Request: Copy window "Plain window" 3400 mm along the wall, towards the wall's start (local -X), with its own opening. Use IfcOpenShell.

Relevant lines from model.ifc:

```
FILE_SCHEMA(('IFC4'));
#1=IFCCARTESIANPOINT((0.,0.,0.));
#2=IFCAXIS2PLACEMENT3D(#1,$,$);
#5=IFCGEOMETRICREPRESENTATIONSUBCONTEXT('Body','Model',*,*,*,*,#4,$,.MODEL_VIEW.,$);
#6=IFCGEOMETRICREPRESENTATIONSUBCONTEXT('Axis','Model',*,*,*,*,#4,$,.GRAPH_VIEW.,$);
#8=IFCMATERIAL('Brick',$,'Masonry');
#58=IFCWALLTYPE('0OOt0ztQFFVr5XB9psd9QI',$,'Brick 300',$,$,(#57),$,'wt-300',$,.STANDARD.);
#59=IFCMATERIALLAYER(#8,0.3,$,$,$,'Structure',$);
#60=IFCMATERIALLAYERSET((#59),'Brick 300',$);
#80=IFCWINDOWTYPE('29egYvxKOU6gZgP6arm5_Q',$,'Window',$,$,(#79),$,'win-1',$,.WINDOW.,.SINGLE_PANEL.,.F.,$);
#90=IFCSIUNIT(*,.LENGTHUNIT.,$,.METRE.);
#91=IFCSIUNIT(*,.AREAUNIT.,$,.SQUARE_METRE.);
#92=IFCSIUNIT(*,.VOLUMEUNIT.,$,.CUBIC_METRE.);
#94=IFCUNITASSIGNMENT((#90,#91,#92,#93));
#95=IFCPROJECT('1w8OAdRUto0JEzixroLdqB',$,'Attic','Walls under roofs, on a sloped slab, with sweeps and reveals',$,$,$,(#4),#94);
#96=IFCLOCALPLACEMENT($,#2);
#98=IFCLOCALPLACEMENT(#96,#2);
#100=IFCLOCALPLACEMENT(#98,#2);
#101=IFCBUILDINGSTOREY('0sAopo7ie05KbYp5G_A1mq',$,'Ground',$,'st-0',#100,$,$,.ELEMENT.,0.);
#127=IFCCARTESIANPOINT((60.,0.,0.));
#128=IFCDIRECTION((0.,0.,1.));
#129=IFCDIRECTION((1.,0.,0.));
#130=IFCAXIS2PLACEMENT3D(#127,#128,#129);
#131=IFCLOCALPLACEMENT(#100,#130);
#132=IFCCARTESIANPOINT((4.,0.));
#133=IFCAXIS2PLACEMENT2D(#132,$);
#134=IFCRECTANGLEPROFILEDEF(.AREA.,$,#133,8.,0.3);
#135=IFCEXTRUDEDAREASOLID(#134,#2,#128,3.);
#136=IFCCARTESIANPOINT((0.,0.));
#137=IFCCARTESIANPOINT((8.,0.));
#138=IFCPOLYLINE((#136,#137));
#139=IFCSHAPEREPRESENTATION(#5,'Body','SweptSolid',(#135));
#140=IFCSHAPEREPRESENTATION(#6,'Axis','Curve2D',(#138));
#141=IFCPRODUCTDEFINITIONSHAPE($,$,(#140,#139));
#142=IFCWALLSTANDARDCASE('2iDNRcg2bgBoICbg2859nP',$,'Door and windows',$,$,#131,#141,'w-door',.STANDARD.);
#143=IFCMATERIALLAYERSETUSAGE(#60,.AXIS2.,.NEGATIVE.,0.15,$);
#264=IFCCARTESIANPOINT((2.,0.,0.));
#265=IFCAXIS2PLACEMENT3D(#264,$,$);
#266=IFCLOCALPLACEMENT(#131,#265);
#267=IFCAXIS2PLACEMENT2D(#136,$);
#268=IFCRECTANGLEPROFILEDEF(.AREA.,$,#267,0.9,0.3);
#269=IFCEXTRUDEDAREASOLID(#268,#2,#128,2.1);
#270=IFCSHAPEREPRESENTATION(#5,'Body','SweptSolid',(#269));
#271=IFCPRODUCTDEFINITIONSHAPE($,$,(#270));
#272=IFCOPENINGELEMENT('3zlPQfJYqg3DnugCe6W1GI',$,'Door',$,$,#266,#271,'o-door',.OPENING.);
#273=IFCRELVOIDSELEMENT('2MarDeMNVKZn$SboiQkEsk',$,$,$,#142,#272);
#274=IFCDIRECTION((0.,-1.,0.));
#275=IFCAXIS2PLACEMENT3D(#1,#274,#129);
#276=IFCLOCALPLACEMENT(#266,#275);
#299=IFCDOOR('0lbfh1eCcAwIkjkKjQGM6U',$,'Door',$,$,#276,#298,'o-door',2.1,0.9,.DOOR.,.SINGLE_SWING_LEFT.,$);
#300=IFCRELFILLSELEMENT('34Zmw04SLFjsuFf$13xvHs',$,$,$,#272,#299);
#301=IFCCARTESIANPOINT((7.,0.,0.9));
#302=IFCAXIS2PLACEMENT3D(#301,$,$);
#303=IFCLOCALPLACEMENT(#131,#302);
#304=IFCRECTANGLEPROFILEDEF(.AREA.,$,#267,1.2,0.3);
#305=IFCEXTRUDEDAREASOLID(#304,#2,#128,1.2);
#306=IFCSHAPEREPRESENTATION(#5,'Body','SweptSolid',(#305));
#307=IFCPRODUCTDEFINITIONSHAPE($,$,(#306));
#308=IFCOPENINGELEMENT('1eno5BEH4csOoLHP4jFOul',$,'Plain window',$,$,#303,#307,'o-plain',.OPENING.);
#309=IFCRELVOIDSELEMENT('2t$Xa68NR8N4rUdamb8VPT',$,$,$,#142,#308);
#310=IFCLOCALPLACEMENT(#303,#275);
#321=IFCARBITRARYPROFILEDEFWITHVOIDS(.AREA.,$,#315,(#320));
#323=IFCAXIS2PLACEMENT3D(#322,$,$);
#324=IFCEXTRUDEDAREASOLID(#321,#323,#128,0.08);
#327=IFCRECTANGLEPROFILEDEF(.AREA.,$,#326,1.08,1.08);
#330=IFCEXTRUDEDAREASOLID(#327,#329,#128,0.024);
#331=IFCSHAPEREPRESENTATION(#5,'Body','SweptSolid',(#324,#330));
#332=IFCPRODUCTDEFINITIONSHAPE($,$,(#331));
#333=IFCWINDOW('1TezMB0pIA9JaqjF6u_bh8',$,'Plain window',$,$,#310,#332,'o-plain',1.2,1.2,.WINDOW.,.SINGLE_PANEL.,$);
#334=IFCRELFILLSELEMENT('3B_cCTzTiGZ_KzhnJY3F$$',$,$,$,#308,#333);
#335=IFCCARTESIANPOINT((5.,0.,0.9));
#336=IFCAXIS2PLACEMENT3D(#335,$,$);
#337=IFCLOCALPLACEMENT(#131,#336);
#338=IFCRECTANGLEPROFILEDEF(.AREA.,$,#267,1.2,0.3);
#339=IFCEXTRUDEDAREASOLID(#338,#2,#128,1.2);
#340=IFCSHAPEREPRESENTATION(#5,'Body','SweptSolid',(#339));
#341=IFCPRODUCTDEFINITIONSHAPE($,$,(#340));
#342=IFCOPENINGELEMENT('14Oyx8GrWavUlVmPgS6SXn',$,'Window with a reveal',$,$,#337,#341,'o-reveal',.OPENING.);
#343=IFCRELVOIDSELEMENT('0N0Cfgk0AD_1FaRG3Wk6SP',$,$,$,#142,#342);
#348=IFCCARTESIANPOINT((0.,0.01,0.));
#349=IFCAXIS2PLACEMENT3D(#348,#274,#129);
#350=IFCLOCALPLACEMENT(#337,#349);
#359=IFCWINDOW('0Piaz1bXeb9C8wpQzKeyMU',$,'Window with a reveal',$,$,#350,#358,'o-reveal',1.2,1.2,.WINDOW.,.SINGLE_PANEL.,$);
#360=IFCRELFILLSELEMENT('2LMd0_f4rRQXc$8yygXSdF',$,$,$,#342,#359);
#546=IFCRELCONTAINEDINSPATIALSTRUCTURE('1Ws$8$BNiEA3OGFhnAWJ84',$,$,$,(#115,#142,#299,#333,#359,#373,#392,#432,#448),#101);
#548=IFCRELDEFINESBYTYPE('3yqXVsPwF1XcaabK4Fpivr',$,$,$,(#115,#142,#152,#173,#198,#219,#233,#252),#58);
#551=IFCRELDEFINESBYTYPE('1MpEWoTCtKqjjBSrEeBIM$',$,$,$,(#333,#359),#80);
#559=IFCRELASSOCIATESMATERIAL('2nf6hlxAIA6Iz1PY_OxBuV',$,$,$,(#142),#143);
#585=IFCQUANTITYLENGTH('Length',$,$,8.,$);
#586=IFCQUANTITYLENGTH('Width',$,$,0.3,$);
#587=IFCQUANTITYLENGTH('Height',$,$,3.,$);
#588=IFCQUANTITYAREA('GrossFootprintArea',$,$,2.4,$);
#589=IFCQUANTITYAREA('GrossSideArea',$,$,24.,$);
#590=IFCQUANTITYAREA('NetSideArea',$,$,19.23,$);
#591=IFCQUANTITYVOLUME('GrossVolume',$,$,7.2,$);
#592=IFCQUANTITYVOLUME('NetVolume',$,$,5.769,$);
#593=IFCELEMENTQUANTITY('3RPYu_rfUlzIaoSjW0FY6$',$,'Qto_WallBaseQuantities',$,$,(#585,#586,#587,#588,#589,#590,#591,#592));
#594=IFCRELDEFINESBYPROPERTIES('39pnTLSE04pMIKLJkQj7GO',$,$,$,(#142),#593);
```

```python
import ifcopenshell
import ifcopenshell.api.feature
import ifcopenshell.api.geometry
import ifcopenshell.api.pset
import ifcopenshell.api.root
import ifcopenshell.geom
import ifcopenshell.util.element
import ifcopenshell.util.placement
import ifcopenshell.util.shape
import ifcopenshell.util.unit

model = ifcopenshell.open("model.ifc")
unit_scale = ifcopenshell.util.unit.calculate_unit_scale(model)
area_scale = ifcopenshell.util.unit.calculate_unit_scale(model, "AREAUNIT")
volume_scale = ifcopenshell.util.unit.calculate_unit_scale(model, "VOLUMEUNIT")
settings = ifcopenshell.geom.settings()


def volume(element):
    """Net volume in cubic metres, openings subtracted."""
    shape = ifcopenshell.geom.create_shape(settings, element)
    return ifcopenshell.util.shape.get_volume(shape.geometry)


window = model.by_guid("1TezMB0pIA9JaqjF6u_bh8")
opening = window.FillsVoids[0].RelatingOpeningElement
wall = opening.VoidsElements[0].RelatingBuildingElement
before = volume(wall)
shift = ifcopenshell.util.placement.get_local_placement(wall.ObjectPlacement)[:3, 0] * -3.4 / unit_scale

# copy_class copies the void relationship, type, container and properties, but no geometry.
new_opening = ifcopenshell.api.root.copy_class(model, product=opening)
new_opening.Representation = ifcopenshell.util.element.copy_deep(
    model, opening.Representation, exclude=["IfcGeometricRepresentationContext", "IfcRepresentationMap"]
)
new_opening.Tag = None
new_window = ifcopenshell.api.root.copy_class(model, product=window)
new_window.Representation = ifcopenshell.util.element.copy_deep(
    model, window.Representation, exclude=["IfcGeometricRepresentationContext", "IfcRepresentationMap"]
)
new_window.Tag = None
ifcopenshell.api.feature.add_filling(model, opening=new_opening, element=new_window)

for old, new in ((opening, new_opening), (window, new_window)):
    matrix = ifcopenshell.util.placement.get_local_placement(old.ObjectPlacement)
    matrix[:3, 3] += shift
    ifcopenshell.api.geometry.edit_object_placement(model, product=new, matrix=matrix, is_si=False)

after = volume(wall)
thickness = 0.3  # wall thickness in metres

# Update the wall's stored quantities.
qto = model.by_id(ifcopenshell.util.element.get_pset(wall, "Qto_WallBaseQuantities", should_inherit=False)["id"])
ifcopenshell.api.pset.edit_qto(model, qto=qto, properties={
    "NetSideArea": after / thickness / area_scale,
    "NetVolume": after / volume_scale,
})

print(f"wall volume {before:.3f} -> {after:.3f} m3")

model.write("model_rev.ifc")
```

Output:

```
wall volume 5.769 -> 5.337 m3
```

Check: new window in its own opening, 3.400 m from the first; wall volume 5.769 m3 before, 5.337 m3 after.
